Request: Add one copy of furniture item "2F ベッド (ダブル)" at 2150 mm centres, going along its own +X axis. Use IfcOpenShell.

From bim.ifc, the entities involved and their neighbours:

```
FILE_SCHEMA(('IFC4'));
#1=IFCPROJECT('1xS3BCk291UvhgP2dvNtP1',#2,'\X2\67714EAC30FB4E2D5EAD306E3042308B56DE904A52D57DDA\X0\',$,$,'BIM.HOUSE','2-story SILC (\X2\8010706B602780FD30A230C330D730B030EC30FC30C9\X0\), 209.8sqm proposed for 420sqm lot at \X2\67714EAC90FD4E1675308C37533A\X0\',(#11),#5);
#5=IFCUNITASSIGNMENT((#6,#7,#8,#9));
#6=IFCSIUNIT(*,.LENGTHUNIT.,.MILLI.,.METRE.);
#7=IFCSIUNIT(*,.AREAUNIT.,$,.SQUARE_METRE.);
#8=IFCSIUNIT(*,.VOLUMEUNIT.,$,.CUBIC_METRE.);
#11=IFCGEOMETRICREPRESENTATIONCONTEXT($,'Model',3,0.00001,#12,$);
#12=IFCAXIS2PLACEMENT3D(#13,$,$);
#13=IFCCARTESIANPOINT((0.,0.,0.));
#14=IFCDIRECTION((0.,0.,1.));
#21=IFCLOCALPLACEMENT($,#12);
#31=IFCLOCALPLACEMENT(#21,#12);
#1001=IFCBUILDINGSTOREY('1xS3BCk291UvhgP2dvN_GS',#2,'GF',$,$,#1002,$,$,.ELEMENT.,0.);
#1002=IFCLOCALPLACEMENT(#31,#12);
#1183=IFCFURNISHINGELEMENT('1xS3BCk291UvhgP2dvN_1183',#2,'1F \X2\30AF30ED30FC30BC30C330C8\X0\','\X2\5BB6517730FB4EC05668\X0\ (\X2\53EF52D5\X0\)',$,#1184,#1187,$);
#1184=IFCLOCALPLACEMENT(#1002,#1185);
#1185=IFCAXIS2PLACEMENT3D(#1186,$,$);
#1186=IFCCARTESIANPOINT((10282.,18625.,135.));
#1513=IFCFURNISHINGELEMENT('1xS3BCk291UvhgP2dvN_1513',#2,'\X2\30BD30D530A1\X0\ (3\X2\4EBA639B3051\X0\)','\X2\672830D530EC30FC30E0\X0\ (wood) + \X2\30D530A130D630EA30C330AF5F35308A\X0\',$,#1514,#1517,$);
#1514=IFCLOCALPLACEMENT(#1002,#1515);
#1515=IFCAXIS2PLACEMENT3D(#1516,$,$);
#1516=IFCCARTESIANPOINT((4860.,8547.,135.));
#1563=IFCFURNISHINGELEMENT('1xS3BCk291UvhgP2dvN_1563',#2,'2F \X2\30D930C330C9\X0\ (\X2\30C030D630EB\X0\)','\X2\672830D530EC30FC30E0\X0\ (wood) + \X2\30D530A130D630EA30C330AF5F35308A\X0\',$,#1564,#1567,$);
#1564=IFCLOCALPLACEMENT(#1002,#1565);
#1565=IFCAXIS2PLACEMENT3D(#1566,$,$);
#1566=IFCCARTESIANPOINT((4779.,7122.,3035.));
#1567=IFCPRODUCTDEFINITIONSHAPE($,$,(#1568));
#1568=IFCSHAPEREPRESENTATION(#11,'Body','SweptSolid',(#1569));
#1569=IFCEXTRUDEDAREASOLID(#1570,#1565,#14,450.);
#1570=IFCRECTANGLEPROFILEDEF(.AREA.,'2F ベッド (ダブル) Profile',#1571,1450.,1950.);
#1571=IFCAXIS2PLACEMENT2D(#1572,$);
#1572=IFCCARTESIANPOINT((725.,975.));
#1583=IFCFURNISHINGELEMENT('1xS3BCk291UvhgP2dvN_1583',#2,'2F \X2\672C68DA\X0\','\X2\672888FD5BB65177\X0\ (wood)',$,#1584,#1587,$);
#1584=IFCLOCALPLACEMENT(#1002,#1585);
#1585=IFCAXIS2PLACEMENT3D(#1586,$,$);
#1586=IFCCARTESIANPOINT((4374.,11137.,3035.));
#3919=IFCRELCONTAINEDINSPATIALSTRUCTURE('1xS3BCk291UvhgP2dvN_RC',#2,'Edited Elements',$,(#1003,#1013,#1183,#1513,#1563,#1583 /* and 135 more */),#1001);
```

```python
import ifcopenshell
import ifcopenshell.api.geometry
import ifcopenshell.api.root
import ifcopenshell.util.element
import ifcopenshell.util.placement

model = ifcopenshell.open("bim.ifc")


def reuse_history(source, copy):
    """copy_class also copies each property set's owner history, people and application; keep the originals."""
    for rel in copy.IsDefinedBy:
        if rel.is_a("IfcRelDefinesByProperties") and (history := rel.RelatingPropertyDefinition.OwnerHistory):
            rel.RelatingPropertyDefinition.OwnerHistory = source.OwnerHistory
            ifcopenshell.util.element.remove_deep2(model, history)


source = model.by_id(1563)
base = ifcopenshell.util.placement.get_local_placement(source.ObjectPlacement)
step = base[:3, 0] * 2150.0

for i in range(1, 2):
    copy = ifcopenshell.api.root.copy_class(model, product=source)
    copy.Representation = ifcopenshell.util.element.copy_deep(
        model, source.Representation, exclude=["IfcGeometricRepresentationContext", "IfcRepresentationMap"]
    )
    reuse_history(source, copy)
    matrix = base.copy()
    matrix[:3, 3] += i * step
    print("added at", matrix[:3, 3].round(3) + 0.0)
    ifcopenshell.api.geometry.edit_object_placement(model, product=copy, matrix=matrix, is_si=False)

model.write("bim-out.ifc")
```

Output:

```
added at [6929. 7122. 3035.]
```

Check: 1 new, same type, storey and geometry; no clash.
